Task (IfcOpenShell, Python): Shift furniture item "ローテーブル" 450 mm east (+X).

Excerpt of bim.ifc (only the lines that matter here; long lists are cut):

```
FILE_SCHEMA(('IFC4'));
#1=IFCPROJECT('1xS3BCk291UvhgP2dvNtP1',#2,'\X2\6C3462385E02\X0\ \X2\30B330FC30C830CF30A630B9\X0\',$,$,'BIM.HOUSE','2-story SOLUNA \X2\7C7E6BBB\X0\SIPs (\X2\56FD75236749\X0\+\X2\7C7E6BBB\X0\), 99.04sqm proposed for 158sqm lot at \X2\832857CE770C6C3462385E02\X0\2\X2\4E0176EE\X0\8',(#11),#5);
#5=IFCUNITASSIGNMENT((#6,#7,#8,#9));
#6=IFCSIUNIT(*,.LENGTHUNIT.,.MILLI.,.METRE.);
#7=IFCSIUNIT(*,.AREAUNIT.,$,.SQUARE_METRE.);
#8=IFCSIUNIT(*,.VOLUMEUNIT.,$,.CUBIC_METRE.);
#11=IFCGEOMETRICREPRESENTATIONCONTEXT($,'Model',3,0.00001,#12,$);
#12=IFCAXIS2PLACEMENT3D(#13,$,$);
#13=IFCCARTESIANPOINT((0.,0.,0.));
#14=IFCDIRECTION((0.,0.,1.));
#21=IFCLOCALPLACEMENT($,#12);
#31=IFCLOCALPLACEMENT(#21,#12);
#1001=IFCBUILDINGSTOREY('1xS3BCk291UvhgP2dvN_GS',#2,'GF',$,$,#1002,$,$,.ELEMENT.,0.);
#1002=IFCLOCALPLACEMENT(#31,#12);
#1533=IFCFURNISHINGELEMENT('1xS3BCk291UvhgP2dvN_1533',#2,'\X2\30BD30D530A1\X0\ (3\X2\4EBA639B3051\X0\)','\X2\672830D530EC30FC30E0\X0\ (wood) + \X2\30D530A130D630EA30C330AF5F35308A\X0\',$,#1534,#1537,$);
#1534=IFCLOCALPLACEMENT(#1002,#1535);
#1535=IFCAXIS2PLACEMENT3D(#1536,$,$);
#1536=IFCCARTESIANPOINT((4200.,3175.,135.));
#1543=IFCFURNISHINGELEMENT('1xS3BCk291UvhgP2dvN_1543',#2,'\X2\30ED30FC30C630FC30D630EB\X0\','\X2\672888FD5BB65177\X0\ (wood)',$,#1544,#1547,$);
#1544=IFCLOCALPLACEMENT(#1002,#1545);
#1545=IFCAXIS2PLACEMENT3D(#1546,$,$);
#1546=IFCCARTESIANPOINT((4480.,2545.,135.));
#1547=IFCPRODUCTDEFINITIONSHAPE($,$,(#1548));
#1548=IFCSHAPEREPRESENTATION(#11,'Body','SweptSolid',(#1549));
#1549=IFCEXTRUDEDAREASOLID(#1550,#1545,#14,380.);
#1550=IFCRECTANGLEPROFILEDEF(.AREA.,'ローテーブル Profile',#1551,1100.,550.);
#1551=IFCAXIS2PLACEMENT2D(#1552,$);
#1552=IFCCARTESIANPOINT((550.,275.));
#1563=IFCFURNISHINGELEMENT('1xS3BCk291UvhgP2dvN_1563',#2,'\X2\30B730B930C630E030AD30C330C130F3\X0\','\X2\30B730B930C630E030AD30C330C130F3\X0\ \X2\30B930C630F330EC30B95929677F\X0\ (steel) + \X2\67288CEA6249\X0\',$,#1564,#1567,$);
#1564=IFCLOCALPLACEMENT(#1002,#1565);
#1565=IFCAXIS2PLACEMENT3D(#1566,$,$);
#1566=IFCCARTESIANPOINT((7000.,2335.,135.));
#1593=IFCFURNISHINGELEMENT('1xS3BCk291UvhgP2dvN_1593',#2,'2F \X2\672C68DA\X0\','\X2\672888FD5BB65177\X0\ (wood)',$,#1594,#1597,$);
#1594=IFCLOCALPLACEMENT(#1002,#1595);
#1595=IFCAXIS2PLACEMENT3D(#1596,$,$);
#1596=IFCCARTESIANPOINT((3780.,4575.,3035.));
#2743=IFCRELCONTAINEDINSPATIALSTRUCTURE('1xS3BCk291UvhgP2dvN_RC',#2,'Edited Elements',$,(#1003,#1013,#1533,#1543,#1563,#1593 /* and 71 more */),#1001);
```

```python
import ifcopenshell
import ifcopenshell.api.geometry
import ifcopenshell.util.placement
import ifcopenshell.util.unit

model = ifcopenshell.open("bim.ifc")
unit_scale = ifcopenshell.util.unit.calculate_unit_scale(model)

item = model.by_guid("1xS3BCk291UvhgP2dvN_1543")
matrix = ifcopenshell.util.placement.get_local_placement(item.ObjectPlacement)
matrix[0, 3] += 0.45 / unit_scale
ifcopenshell.api.geometry.edit_object_placement(model, product=item, matrix=matrix, is_si=False)

print(ifcopenshell.util.placement.get_local_placement(item.ObjectPlacement).round(3) + 0.0)

model.write("bim_edited.ifc")
```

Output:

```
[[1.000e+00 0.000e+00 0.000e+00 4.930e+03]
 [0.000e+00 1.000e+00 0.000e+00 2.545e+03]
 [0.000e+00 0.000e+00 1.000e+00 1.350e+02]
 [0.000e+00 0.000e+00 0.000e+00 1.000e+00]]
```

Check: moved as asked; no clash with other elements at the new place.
